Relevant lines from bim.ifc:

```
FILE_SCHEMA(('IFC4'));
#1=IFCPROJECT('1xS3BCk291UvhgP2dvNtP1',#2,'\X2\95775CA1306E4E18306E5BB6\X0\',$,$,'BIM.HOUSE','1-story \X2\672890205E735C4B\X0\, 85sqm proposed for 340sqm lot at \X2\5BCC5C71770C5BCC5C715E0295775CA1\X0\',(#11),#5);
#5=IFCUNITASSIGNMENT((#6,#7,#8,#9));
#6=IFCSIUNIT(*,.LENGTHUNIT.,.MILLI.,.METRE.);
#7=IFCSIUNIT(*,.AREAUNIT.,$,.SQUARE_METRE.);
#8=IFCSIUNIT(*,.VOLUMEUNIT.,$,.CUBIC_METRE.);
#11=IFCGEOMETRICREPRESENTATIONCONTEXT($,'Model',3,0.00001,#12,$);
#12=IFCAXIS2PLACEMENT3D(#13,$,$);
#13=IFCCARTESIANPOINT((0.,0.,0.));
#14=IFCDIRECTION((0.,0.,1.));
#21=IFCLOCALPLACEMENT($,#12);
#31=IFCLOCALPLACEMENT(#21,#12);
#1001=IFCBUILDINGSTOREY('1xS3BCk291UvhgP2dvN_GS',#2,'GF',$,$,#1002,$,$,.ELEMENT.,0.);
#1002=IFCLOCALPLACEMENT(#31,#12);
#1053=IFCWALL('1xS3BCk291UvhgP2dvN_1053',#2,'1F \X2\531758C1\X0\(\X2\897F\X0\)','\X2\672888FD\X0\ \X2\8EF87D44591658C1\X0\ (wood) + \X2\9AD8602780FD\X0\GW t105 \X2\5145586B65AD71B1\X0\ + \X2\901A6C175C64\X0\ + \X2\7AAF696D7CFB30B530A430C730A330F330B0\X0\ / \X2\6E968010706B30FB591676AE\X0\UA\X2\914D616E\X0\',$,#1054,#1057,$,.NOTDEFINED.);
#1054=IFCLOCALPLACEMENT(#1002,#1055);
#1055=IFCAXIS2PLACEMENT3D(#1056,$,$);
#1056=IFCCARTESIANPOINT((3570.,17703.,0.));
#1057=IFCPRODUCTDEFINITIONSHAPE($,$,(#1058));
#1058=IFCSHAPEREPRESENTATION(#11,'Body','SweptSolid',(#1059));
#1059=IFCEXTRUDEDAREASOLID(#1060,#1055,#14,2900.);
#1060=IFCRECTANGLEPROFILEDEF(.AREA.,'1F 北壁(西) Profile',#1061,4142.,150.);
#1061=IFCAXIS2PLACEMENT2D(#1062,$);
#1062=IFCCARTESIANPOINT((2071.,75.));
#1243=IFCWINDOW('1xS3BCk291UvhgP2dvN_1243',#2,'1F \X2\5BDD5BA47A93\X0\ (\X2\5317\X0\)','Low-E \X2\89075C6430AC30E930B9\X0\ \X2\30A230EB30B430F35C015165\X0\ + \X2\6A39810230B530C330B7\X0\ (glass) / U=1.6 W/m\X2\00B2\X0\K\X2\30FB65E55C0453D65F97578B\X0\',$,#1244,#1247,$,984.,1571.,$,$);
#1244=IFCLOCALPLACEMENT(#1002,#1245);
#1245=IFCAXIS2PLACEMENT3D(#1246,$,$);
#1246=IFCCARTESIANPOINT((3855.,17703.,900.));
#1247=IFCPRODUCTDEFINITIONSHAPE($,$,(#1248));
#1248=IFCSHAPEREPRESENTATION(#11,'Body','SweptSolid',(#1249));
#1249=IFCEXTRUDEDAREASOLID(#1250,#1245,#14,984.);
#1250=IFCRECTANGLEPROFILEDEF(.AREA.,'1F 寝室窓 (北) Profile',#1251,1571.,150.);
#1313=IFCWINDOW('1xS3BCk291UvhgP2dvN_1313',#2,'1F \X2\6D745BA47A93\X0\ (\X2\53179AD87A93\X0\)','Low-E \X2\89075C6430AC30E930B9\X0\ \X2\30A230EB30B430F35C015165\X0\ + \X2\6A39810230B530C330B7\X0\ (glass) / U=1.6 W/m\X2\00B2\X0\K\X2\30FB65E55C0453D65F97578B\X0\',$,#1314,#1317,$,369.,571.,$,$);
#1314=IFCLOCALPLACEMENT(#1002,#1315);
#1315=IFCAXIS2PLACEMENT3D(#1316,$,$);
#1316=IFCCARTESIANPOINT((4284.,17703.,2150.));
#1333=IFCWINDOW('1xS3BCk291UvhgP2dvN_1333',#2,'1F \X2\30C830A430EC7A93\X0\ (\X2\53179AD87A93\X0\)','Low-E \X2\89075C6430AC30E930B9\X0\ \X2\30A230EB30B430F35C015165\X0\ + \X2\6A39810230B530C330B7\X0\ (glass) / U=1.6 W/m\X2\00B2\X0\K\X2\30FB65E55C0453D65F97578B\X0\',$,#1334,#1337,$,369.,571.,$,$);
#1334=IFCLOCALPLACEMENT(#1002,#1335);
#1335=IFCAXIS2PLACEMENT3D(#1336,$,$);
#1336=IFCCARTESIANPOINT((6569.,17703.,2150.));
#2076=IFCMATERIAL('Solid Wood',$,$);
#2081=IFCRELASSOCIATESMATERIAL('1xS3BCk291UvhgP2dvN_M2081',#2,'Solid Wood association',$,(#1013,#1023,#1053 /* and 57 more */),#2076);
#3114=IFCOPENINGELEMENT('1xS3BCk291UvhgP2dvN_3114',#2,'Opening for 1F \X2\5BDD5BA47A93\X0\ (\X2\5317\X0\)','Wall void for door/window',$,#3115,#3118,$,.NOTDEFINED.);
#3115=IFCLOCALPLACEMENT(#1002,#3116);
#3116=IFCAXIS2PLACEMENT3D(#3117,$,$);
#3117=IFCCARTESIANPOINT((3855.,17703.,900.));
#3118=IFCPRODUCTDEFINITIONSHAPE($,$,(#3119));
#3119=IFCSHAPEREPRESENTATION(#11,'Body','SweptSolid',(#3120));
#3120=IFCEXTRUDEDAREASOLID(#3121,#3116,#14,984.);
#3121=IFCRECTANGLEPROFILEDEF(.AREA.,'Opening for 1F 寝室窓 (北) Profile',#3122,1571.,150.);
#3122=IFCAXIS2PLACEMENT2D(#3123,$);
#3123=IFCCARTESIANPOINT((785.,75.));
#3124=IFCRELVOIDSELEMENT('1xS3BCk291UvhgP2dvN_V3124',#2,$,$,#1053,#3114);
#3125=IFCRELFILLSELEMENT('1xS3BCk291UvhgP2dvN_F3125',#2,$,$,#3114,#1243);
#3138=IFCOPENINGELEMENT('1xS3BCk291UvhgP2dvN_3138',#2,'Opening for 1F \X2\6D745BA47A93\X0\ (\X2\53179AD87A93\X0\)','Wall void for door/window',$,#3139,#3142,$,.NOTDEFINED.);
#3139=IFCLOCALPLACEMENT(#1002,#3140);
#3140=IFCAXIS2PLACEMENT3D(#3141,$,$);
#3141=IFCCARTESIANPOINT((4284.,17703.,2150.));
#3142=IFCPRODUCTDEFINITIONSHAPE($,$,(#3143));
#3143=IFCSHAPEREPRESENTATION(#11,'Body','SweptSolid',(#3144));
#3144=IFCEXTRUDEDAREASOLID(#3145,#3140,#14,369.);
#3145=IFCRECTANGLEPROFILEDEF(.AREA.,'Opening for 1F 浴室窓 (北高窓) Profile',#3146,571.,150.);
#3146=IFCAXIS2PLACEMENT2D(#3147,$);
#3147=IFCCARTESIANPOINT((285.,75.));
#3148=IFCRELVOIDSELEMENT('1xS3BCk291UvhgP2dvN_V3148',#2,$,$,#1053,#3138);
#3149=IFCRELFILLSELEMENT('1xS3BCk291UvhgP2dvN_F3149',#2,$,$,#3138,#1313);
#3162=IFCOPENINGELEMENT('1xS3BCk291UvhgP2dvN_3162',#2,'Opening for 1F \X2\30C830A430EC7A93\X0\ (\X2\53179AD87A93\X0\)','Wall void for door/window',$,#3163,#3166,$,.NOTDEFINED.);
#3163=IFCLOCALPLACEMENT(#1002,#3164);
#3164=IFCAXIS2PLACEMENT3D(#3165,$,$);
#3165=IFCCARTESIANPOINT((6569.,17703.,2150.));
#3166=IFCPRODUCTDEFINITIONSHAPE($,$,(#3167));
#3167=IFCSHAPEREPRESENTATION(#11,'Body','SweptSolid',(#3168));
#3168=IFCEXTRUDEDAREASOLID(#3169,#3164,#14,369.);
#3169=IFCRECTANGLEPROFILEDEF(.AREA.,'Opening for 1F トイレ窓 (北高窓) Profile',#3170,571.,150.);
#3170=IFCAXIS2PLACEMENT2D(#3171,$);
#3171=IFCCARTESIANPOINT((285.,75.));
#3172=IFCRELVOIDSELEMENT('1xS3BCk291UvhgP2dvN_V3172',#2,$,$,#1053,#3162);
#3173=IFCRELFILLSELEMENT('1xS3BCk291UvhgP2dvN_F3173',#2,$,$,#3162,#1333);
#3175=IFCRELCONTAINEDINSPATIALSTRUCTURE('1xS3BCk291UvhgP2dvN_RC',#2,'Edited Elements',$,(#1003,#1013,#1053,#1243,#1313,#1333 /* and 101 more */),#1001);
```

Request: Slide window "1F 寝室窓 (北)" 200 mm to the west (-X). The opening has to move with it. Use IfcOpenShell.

```python
import ifcopenshell
import ifcopenshell.api.geometry
import ifcopenshell.util.placement
import ifcopenshell.util.unit

model = ifcopenshell.open("bim.ifc")
unit_scale = ifcopenshell.util.unit.calculate_unit_scale(model)

window = model.by_id(1243)
opening = window.FillsVoids[0].RelatingOpeningElement
wall = opening.VoidsElements[0].RelatingBuildingElement

wall_matrix = ifcopenshell.util.placement.get_local_placement(wall.ObjectPlacement)
shift = wall_matrix[:3, 0] * -0.2 / unit_scale
before = ifcopenshell.util.placement.get_local_placement(window.ObjectPlacement)[:3, 3].copy()

# The window is not placed relative to its opening, so move both.
for product in (opening, window):
    matrix = ifcopenshell.util.placement.get_local_placement(product.ObjectPlacement)
    matrix[:3, 3] += shift
    ifcopenshell.api.geometry.edit_object_placement(model, product=product, matrix=matrix, is_si=False)

after = ifcopenshell.util.placement.get_local_placement(window.ObjectPlacement)[:3, 3]
print("window moved by", (after - before).round(3) + 0.0)

model.write("bim_rev.ifc")
```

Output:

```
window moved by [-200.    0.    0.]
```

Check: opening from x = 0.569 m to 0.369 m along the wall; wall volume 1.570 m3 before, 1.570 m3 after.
